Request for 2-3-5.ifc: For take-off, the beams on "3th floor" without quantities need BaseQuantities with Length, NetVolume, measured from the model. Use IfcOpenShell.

First a look at what the model holds.

```python
import ifcopenshell
import ifcopenshell.util.element
import ifcopenshell.util.unit

model = ifcopenshell.open("2-3-5.ifc")
print(model.schema)
for unit_type in ("LENGTHUNIT", "AREAUNIT", "VOLUMEUNIT"):
    print(unit_type, ifcopenshell.util.unit.calculate_unit_scale(model, unit_type))
storey = next(s for s in model.by_type("IfcBuildingStorey") if s.Name == "3th floor")
beams = [e for e in ifcopenshell.util.element.get_decomposition(storey) if e.is_a("IfcBeam")]
for e in sorted(beams, key=lambda e: e.id()):
    print(e.id(), e.is_a(), e.Name, list(ifcopenshell.util.element.get_psets(e, qtos_only=True)), sep=" | ")
```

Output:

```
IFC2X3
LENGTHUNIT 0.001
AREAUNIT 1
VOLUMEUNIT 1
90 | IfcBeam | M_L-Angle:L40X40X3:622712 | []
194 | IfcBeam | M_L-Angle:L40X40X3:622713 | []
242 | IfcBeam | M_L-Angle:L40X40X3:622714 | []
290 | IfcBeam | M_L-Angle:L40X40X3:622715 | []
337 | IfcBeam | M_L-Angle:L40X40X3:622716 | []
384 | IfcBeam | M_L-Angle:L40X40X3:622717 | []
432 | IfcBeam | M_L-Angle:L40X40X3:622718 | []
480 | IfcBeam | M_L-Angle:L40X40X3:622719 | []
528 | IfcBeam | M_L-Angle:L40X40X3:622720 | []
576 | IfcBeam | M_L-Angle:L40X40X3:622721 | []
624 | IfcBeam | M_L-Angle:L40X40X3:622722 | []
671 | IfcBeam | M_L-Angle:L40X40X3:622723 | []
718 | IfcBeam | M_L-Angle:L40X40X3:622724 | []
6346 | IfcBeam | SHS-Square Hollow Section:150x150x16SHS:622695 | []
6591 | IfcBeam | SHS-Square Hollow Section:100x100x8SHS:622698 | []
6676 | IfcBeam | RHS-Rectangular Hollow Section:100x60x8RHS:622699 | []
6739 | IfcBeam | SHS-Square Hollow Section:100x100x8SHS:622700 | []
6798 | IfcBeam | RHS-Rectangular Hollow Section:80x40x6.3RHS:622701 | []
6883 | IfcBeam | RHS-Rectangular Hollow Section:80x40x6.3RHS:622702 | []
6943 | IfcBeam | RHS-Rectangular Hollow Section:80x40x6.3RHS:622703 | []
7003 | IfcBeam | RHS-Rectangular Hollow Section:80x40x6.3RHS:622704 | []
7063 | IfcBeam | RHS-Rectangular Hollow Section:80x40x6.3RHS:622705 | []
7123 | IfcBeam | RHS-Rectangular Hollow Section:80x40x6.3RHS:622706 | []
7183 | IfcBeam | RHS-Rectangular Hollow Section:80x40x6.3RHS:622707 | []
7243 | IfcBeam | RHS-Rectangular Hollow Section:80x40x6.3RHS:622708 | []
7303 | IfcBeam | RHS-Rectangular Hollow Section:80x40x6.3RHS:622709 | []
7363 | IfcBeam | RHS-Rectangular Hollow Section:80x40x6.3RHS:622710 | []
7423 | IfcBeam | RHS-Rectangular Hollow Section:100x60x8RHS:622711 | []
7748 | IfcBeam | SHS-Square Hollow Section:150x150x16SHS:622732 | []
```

```python
import ifcopenshell
import ifcopenshell.api.pset
import ifcopenshell.geom
import ifcopenshell.util.element
import ifcopenshell.util.shape
import ifcopenshell.util.unit

model = ifcopenshell.open("2-3-5.ifc")
unit_scale = ifcopenshell.util.unit.calculate_unit_scale(model)
volume_scale = ifcopenshell.util.unit.calculate_unit_scale(model, "VOLUMEUNIT")
settings = ifcopenshell.geom.settings()

storey = next(s for s in model.by_type("IfcBuildingStorey") if s.Name == "3th floor")
beams = [e for e in ifcopenshell.util.element.get_decomposition(storey) if e.is_a("IfcBeam")]

for e in sorted(beams, key=lambda e: e.id()):
    if ifcopenshell.util.element.get_psets(e, qtos_only=True, should_inherit=False):
        continue
    # Geometry comes back in metres, in the element's own axes.
    shape = ifcopenshell.geom.create_shape(settings, e)
    values = {
        "Length": ifcopenshell.util.shape.get_max_xyz(shape.geometry) / unit_scale,
        "NetVolume": ifcopenshell.util.shape.get_volume(shape.geometry) / volume_scale,
    }
    qto = ifcopenshell.api.pset.add_qto(model, product=e, name="BaseQuantities")
    ifcopenshell.api.pset.edit_qto(model, qto=qto, properties=values)
    print(e.id(), {k: round(v, 3) for k, v in values.items()})

model.write("2-3-5-out.ifc")
```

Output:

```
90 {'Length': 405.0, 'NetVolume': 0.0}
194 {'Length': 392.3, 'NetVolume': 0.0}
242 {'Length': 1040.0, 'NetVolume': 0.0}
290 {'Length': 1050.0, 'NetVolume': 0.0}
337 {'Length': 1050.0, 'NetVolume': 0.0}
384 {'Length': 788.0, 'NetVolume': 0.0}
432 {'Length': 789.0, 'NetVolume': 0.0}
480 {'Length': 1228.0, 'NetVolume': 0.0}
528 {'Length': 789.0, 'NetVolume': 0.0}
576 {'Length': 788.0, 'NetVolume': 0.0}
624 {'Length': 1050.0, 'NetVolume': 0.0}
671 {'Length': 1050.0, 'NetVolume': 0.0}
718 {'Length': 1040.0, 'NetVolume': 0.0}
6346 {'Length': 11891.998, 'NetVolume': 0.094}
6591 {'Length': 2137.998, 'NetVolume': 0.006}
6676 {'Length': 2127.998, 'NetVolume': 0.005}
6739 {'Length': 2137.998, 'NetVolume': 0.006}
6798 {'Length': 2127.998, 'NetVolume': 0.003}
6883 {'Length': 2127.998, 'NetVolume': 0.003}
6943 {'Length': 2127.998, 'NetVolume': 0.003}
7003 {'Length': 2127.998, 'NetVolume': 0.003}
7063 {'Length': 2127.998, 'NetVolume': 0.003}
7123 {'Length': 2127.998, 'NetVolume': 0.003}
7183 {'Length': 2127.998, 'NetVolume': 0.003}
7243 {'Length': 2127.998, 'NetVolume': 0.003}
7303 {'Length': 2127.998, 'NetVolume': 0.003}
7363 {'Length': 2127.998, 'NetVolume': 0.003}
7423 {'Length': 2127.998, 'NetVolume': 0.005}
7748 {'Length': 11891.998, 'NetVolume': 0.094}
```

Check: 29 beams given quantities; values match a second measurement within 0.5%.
